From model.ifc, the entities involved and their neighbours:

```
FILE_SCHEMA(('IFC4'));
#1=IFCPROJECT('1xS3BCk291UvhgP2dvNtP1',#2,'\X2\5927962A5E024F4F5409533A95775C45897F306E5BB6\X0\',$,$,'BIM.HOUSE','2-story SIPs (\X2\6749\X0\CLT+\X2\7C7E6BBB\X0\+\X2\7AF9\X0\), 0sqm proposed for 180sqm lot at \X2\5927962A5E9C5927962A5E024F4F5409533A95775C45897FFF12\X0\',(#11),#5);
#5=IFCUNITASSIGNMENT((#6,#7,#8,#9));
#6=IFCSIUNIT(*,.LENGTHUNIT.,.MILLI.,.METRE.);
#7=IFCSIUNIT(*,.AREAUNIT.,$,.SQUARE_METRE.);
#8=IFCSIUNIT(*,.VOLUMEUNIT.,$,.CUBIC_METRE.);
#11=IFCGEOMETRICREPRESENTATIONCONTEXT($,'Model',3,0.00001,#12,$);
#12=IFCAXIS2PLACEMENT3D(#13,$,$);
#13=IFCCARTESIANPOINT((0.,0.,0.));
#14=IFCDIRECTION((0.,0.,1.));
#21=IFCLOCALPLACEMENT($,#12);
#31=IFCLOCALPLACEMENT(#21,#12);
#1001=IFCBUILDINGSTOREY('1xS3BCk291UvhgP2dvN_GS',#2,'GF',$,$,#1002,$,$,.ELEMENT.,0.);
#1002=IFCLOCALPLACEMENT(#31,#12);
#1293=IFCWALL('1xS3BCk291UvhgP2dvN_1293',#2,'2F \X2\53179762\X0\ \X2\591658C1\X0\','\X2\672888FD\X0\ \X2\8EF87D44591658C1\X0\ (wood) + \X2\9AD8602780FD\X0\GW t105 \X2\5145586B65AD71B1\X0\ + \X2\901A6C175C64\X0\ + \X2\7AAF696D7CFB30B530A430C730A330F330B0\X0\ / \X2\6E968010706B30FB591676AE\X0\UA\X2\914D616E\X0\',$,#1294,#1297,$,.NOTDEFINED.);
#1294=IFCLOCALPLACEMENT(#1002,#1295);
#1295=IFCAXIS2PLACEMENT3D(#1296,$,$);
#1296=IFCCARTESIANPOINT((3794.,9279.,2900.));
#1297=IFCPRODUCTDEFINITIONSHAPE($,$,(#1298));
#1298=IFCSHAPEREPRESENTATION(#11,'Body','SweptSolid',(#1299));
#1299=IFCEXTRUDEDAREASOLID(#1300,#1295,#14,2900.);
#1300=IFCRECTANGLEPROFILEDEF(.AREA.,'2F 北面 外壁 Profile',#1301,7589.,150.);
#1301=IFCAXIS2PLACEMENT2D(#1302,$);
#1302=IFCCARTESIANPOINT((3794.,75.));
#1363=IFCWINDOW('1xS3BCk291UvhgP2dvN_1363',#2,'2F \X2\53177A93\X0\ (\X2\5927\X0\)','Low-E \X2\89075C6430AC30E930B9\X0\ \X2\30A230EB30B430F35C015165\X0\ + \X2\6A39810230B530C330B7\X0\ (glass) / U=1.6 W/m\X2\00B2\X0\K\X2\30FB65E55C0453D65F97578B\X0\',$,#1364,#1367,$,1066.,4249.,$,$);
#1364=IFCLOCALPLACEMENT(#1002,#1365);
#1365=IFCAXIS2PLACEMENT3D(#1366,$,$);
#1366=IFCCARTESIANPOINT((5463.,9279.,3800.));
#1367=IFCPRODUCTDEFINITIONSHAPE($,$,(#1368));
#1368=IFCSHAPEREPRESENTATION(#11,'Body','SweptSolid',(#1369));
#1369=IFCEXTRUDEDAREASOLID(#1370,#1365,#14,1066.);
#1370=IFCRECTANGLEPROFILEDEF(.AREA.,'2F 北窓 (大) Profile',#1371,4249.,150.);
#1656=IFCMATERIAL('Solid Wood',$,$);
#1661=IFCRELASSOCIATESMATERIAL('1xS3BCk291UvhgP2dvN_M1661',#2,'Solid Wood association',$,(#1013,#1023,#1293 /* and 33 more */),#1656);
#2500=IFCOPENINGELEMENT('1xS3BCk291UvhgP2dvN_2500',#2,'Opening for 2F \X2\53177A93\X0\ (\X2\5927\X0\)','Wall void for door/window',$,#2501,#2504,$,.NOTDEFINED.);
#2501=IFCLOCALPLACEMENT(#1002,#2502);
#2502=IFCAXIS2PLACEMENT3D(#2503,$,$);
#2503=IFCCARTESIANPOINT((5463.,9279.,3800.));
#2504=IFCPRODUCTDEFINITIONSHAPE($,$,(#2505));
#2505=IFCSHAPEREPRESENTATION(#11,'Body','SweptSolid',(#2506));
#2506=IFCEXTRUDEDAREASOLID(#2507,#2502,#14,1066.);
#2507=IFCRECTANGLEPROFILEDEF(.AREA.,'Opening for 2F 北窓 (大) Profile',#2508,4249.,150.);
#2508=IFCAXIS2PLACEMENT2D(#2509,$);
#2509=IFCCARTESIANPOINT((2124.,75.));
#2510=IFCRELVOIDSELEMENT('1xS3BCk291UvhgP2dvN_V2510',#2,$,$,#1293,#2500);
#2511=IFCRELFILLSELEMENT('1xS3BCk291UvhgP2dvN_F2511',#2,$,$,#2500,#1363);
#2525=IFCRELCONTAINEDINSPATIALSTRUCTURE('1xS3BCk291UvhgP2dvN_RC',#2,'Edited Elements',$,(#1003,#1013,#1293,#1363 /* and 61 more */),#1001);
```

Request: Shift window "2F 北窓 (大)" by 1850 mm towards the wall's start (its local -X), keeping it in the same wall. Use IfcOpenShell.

```python
import ifcopenshell
import ifcopenshell.api.geometry
import ifcopenshell.util.placement

model = ifcopenshell.open("model.ifc")

window = model.by_guid("1xS3BCk291UvhgP2dvN_1363")
opening = window.FillsVoids[0].RelatingOpeningElement
wall = opening.VoidsElements[0].RelatingBuildingElement

wall_matrix = ifcopenshell.util.placement.get_local_placement(wall.ObjectPlacement)
shift = wall_matrix[:3, 0] * -1850.0
before = ifcopenshell.util.placement.get_local_placement(window.ObjectPlacement)[:3, 3].copy()

# The window is not placed relative to its opening, so move both.
for product in (opening, window):
    matrix = ifcopenshell.util.placement.get_local_placement(product.ObjectPlacement)
    matrix[:3, 3] += shift
    ifcopenshell.api.geometry.edit_object_placement(model, product=product, matrix=matrix, is_si=False)

after = ifcopenshell.util.placement.get_local_placement(window.ObjectPlacement)[:3, 3]
print("window moved by", (after - before).round(3) + 0.0)

model.write("model_edited.ifc")
```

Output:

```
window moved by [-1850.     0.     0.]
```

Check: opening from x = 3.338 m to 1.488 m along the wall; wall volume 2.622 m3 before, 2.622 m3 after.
